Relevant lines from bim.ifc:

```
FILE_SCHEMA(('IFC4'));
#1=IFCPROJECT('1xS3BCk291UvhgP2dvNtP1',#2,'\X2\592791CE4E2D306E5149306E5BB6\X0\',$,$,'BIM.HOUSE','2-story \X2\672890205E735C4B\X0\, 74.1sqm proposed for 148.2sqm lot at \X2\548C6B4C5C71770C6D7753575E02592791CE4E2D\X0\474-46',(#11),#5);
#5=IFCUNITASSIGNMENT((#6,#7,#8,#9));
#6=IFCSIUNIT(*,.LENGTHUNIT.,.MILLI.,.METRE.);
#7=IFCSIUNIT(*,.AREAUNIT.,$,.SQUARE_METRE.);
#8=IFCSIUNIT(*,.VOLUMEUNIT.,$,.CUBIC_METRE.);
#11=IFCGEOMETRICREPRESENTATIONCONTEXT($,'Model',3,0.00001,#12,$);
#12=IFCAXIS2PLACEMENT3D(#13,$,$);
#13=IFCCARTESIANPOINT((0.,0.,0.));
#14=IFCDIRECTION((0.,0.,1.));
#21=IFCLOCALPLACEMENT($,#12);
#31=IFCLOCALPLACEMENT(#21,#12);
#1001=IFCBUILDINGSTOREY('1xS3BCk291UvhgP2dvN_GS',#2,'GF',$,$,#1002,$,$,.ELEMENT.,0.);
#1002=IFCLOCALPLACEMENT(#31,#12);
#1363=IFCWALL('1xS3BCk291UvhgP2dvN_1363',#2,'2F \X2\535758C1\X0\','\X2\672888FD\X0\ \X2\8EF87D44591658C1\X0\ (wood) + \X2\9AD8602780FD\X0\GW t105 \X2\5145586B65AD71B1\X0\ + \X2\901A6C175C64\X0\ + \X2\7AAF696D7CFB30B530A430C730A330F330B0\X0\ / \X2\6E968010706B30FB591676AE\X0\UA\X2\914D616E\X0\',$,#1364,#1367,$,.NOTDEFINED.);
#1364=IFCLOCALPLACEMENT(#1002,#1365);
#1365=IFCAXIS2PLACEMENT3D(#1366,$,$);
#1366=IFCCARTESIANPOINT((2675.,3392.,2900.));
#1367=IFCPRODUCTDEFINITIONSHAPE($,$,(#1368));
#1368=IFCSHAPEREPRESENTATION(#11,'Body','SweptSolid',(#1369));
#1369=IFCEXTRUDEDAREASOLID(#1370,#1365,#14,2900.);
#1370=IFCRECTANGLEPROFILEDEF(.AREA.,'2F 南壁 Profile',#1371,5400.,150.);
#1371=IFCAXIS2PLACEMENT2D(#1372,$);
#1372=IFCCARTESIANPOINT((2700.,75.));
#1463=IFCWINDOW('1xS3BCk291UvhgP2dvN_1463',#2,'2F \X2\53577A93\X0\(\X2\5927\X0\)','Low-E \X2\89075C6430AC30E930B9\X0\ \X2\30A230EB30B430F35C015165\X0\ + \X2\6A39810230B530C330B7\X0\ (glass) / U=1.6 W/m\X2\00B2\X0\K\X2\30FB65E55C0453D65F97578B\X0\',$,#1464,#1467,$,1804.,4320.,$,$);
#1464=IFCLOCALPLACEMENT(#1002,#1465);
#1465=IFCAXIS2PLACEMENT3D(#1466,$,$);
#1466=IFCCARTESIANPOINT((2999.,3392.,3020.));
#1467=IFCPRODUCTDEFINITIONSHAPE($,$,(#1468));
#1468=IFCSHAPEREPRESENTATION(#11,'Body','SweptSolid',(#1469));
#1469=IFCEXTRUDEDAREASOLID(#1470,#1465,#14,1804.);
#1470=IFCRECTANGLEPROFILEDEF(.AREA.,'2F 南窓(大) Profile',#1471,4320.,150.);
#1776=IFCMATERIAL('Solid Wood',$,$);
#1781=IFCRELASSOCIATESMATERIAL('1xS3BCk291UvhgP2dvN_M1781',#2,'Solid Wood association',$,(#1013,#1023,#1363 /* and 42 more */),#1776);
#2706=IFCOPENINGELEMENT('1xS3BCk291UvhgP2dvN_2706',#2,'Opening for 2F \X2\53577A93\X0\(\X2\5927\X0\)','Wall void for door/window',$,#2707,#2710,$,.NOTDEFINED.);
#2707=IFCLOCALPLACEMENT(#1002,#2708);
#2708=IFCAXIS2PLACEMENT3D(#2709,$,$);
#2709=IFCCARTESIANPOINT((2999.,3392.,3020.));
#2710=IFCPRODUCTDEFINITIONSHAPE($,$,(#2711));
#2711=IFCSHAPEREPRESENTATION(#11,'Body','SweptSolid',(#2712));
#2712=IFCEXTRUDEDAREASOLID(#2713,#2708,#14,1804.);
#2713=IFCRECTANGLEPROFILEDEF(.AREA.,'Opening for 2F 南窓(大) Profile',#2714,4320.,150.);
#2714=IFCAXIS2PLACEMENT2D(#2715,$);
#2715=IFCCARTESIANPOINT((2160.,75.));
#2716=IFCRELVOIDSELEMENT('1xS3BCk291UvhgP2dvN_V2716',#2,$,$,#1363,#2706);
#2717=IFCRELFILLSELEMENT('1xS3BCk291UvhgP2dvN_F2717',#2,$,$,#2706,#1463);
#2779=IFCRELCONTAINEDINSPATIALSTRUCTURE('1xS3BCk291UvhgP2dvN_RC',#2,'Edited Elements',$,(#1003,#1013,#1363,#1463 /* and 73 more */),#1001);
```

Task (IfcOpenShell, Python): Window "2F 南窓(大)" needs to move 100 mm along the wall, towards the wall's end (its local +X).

```python
import ifcopenshell
import ifcopenshell.api.geometry
import ifcopenshell.util.placement
import ifcopenshell.util.unit

model = ifcopenshell.open("bim.ifc")
unit_scale = ifcopenshell.util.unit.calculate_unit_scale(model)

window = model.by_guid("1xS3BCk291UvhgP2dvN_1463")
opening = window.FillsVoids[0].RelatingOpeningElement
wall = opening.VoidsElements[0].RelatingBuildingElement

wall_matrix = ifcopenshell.util.placement.get_local_placement(wall.ObjectPlacement)
shift = wall_matrix[:3, 0] * 0.1 / unit_scale
before = ifcopenshell.util.placement.get_local_placement(window.ObjectPlacement)[:3, 3].copy()

# The window is not placed relative to its opening, so move both.
for product in (opening, window):
    matrix = ifcopenshell.util.placement.get_local_placement(product.ObjectPlacement)
    matrix[:3, 3] += shift
    ifcopenshell.api.geometry.edit_object_placement(model, product=product, matrix=matrix, is_si=False)

after = ifcopenshell.util.placement.get_local_placement(window.ObjectPlacement)[:3, 3]
print("window moved by", (after - before).round(3) + 0.0)

model.write("bim_rev.ifc")
```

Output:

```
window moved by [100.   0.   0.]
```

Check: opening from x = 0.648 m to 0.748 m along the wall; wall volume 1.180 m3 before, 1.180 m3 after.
